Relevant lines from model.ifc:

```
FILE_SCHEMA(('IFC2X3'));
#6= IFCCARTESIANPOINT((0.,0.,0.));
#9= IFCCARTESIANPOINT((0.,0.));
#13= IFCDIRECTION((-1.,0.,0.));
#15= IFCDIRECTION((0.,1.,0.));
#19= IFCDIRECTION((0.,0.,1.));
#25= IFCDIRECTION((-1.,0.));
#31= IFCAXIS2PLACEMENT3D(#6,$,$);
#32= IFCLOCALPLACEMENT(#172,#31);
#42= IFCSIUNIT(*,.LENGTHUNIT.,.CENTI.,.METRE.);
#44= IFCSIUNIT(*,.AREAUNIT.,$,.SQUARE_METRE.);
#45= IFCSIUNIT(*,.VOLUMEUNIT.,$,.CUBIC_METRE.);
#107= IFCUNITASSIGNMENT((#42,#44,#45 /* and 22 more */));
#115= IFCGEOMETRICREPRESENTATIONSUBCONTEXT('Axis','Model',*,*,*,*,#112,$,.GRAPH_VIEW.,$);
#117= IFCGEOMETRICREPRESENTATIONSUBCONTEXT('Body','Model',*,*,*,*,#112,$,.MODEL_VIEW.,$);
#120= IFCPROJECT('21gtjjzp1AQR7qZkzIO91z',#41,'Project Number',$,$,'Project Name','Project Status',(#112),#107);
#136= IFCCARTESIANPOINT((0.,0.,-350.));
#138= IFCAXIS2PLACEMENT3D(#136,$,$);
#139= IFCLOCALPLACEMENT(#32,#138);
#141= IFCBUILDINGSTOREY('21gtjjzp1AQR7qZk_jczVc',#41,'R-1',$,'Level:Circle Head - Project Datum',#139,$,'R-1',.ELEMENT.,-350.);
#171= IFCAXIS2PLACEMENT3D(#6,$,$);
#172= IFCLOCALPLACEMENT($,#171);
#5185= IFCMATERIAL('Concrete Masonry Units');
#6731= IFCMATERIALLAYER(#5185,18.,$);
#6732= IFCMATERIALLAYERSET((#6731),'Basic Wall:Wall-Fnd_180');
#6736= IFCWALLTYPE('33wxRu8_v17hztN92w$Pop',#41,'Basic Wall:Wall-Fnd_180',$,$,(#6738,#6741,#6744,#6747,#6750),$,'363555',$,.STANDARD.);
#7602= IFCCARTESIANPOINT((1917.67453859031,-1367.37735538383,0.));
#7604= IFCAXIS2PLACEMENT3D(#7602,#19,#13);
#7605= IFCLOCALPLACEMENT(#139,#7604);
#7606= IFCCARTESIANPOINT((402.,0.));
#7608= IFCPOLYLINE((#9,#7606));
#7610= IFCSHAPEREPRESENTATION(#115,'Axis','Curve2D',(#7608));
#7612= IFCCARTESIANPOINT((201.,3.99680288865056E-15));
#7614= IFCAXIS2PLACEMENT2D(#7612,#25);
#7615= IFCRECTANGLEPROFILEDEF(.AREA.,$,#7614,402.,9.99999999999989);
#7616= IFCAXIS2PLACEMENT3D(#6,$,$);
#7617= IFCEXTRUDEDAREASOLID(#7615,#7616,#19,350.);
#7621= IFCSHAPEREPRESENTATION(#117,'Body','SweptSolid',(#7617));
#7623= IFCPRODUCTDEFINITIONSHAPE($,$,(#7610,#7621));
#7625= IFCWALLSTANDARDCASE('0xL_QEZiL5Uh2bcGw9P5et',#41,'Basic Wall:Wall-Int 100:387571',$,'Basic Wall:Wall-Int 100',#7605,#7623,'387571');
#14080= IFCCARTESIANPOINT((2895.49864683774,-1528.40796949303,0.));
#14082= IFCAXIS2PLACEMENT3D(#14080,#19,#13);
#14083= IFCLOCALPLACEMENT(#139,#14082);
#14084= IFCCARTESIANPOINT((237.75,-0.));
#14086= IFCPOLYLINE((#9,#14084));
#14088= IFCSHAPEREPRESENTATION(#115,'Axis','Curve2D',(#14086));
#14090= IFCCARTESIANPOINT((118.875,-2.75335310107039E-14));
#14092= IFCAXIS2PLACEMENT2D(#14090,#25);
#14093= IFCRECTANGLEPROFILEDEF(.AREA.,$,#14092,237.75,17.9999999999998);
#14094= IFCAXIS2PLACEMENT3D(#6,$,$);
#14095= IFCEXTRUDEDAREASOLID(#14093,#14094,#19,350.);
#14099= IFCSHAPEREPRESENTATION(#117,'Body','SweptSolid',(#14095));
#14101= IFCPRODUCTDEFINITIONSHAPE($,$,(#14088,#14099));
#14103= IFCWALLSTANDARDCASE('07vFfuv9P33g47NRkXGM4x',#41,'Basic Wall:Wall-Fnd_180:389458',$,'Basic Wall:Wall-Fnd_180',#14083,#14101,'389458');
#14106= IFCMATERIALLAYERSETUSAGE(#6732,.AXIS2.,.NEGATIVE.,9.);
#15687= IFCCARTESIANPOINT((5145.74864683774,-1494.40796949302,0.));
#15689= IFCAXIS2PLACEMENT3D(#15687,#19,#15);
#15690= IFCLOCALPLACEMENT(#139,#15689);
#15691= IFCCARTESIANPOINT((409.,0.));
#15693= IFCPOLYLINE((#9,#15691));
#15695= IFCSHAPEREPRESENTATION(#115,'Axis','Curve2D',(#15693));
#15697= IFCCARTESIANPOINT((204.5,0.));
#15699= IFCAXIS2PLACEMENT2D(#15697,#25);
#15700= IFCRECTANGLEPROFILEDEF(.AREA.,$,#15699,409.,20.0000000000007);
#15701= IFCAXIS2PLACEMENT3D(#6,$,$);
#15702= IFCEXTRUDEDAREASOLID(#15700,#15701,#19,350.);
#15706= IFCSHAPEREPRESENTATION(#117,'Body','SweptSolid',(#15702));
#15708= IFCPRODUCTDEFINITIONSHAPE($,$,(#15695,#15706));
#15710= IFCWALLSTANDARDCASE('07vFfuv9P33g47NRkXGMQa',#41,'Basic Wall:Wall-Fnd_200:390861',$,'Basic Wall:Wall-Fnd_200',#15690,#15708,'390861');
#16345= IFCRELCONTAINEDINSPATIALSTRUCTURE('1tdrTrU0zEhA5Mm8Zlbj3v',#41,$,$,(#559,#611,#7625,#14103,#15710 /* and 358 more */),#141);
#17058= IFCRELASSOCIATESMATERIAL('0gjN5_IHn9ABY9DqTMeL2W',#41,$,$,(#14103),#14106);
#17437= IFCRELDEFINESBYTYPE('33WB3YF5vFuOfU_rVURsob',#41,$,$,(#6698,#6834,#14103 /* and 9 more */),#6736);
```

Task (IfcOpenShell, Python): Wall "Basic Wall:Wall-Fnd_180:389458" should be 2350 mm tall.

```python
import ifcopenshell
import ifcopenshell.geom
import ifcopenshell.util.representation
import ifcopenshell.util.shape
import ifcopenshell.util.unit

model = ifcopenshell.open("model.ifc")
unit_scale = ifcopenshell.util.unit.calculate_unit_scale(model)
settings = ifcopenshell.geom.settings()


def volume(element):
    """Net volume in cubic metres, openings subtracted."""
    shape = ifcopenshell.geom.create_shape(settings, element)
    return ifcopenshell.util.shape.get_volume(shape.geometry)


wall = model.by_guid("07vFfuv9P33g47NRkXGM4x")
before = volume(wall)

body = ifcopenshell.util.representation.get_representation(wall, "Model", "Body")
solid = body.Items[0]
old_height = solid.Depth
solid.Depth = 2.35 / unit_scale
after = volume(wall)

print(f"height {old_height:g} -> {solid.Depth:g}, volume {before:.3f} -> {after:.3f} m3")

model.write("model_edited.ifc")
```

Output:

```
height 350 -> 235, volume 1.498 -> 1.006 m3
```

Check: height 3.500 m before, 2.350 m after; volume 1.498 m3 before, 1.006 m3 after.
